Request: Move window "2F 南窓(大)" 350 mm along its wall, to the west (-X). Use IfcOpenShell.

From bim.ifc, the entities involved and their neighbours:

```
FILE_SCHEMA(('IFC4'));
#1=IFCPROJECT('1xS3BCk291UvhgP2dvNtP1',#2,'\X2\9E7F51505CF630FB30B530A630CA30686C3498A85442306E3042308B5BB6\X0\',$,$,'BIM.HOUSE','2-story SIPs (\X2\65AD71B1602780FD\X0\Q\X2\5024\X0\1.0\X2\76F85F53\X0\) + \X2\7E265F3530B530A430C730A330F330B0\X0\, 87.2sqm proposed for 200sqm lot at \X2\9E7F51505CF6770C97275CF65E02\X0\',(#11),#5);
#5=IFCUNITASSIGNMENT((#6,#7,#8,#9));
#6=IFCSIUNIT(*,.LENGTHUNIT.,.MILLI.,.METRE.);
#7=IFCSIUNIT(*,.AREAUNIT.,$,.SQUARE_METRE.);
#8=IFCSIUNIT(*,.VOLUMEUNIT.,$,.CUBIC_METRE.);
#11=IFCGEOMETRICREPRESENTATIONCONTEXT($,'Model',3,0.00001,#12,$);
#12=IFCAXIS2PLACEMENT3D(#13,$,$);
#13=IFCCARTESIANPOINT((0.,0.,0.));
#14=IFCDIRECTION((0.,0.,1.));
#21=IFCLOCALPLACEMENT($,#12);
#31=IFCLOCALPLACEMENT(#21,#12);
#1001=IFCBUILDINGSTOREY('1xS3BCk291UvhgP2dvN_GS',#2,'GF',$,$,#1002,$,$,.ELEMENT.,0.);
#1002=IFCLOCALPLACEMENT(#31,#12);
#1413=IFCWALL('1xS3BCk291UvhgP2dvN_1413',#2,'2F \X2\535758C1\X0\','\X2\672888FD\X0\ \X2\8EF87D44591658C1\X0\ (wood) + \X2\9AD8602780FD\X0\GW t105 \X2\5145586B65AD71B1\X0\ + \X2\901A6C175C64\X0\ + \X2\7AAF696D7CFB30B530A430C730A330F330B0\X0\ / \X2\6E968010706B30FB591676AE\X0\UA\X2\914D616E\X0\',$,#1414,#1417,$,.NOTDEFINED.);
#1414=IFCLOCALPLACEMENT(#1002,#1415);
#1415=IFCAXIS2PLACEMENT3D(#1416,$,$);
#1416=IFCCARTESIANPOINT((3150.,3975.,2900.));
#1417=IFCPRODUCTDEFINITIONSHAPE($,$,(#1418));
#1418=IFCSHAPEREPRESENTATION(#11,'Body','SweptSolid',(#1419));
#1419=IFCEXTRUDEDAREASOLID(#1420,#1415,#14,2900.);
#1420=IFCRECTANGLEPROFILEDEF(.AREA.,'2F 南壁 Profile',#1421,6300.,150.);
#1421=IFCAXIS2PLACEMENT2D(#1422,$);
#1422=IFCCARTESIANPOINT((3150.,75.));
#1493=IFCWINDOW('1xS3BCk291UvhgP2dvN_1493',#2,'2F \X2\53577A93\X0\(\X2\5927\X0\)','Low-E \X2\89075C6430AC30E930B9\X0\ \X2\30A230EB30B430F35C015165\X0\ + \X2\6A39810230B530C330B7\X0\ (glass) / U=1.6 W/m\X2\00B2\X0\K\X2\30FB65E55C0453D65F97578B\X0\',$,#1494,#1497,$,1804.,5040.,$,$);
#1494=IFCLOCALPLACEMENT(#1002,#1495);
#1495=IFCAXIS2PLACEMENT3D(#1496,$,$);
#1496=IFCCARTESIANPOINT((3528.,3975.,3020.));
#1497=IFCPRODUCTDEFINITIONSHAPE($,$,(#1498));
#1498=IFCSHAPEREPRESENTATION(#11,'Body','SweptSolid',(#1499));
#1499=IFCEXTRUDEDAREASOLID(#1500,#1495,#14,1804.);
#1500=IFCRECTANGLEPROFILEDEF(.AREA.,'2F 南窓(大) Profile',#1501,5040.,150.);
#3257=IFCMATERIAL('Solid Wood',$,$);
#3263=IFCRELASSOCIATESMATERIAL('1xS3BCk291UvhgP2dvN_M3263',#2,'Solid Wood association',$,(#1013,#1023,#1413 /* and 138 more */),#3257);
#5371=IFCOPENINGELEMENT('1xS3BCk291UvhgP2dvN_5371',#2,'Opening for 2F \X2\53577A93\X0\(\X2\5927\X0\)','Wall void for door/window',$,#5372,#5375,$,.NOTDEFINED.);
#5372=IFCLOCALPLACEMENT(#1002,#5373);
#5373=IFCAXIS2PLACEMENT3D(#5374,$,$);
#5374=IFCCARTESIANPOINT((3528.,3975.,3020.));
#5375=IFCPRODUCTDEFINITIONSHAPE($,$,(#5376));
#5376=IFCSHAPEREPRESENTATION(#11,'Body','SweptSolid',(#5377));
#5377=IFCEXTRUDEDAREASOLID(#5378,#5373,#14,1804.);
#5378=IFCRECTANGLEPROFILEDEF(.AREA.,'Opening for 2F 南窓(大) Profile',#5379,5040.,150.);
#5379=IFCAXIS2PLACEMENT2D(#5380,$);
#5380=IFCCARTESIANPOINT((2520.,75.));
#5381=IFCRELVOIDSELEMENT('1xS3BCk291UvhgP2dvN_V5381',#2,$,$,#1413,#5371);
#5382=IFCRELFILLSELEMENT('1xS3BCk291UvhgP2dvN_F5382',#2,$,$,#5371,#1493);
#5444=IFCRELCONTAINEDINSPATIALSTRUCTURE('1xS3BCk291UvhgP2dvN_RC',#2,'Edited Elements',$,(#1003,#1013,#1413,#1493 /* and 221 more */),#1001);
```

```python
import ifcopenshell
import ifcopenshell.api.geometry
import ifcopenshell.util.placement

model = ifcopenshell.open("bim.ifc")

window = model.by_id(1493)
opening = window.FillsVoids[0].RelatingOpeningElement
wall = opening.VoidsElements[0].RelatingBuildingElement

wall_matrix = ifcopenshell.util.placement.get_local_placement(wall.ObjectPlacement)
shift = wall_matrix[:3, 0] * -350.0
before = ifcopenshell.util.placement.get_local_placement(window.ObjectPlacement)[:3, 3].copy()

# The window is not placed relative to its opening, so move both.
for product in (opening, window):
    matrix = ifcopenshell.util.placement.get_local_placement(product.ObjectPlacement)
    matrix[:3, 3] += shift
    ifcopenshell.api.geometry.edit_object_placement(model, product=product, matrix=matrix, is_si=False)

after = ifcopenshell.util.placement.get_local_placement(window.ObjectPlacement)[:3, 3]
print("window moved by", (after - before).round(3) + 0.0)

model.write("bim_v2.ifc")
```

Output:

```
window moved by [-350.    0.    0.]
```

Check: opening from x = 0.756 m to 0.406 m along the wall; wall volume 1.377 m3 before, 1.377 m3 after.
